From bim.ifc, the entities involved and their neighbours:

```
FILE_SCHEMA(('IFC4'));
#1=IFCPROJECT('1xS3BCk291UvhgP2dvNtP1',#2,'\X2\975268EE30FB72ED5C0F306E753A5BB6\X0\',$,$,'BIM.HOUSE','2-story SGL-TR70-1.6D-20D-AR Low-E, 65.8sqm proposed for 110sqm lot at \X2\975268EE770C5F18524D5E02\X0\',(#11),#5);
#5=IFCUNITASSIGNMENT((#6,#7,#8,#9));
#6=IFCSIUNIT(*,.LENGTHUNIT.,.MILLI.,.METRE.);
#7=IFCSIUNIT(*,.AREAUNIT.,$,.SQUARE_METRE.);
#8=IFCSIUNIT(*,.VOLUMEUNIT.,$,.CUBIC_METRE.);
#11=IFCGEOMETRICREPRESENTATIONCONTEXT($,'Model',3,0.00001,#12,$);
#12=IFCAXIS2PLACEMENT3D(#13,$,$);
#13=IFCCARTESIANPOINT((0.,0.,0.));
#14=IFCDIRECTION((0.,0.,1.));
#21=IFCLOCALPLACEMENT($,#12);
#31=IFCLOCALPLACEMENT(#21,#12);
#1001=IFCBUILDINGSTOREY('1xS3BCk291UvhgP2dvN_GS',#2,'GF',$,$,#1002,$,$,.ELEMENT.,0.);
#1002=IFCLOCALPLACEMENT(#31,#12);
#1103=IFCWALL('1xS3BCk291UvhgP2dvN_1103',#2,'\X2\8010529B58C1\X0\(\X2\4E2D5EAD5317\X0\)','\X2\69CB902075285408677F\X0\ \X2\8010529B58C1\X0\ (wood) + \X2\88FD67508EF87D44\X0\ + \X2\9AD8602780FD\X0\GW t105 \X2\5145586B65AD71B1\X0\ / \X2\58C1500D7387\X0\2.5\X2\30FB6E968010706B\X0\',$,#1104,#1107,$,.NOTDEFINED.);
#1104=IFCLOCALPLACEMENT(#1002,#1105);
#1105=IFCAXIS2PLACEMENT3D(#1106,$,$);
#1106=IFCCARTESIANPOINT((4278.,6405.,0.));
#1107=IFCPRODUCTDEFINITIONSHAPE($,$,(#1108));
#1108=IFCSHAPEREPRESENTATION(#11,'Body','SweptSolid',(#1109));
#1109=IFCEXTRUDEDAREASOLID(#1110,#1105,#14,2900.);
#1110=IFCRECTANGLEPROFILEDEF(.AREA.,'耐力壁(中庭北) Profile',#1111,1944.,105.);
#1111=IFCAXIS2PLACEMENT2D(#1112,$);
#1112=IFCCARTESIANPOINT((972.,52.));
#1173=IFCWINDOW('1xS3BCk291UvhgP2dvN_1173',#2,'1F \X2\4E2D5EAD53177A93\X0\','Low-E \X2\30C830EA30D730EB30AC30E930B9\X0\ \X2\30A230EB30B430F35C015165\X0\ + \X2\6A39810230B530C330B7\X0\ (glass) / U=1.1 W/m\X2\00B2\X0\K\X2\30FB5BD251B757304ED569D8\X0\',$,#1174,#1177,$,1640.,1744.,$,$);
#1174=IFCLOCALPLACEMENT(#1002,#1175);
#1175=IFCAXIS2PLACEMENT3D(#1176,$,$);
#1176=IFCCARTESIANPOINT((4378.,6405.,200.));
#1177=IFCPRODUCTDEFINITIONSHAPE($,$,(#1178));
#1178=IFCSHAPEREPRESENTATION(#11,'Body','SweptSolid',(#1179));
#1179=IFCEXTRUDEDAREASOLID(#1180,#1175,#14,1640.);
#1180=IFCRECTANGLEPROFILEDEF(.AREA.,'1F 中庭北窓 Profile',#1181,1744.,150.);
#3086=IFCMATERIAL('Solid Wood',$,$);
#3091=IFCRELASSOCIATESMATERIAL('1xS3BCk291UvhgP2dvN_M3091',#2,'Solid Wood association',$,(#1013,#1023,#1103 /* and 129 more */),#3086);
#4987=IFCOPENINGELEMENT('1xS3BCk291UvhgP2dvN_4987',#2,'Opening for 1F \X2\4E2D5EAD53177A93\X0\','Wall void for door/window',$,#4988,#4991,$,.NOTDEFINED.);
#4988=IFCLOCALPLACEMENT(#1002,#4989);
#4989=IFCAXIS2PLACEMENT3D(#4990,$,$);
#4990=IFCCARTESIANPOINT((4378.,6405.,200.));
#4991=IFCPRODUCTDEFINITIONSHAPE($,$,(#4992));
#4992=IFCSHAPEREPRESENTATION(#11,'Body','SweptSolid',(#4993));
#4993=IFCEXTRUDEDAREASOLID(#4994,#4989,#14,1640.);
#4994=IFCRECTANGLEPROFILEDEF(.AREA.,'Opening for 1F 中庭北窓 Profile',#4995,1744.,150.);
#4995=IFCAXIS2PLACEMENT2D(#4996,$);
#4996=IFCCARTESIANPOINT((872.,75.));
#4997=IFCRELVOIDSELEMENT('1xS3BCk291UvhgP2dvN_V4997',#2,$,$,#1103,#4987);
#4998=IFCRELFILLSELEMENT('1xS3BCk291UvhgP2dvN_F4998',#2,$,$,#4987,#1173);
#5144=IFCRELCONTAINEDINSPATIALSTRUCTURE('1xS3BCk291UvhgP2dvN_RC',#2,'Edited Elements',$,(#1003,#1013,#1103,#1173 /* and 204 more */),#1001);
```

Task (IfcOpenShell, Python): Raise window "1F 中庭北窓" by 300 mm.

```python
import numpy as np
import ifcopenshell
import ifcopenshell.api.geometry
import ifcopenshell.util.placement
import ifcopenshell.util.unit

model = ifcopenshell.open("bim.ifc")
unit_scale = ifcopenshell.util.unit.calculate_unit_scale(model)

window = model.by_guid("1xS3BCk291UvhgP2dvN_1173")
opening = window.FillsVoids[0].RelatingOpeningElement
dz = 0.3 / unit_scale

shift = np.array([0.0, 0.0, dz])
# The window is not placed relative to its opening, so move both.
for product in (opening, window):
    matrix = ifcopenshell.util.placement.get_local_placement(product.ObjectPlacement)
    matrix[:3, 3] += shift
    ifcopenshell.api.geometry.edit_object_placement(model, product=product, matrix=matrix, is_si=False)

print(f"moved by {dz * unit_scale:+.3f} m")

model.write("bim_edited.ifc")
```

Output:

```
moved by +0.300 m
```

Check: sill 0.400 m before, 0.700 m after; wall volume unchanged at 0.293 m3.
